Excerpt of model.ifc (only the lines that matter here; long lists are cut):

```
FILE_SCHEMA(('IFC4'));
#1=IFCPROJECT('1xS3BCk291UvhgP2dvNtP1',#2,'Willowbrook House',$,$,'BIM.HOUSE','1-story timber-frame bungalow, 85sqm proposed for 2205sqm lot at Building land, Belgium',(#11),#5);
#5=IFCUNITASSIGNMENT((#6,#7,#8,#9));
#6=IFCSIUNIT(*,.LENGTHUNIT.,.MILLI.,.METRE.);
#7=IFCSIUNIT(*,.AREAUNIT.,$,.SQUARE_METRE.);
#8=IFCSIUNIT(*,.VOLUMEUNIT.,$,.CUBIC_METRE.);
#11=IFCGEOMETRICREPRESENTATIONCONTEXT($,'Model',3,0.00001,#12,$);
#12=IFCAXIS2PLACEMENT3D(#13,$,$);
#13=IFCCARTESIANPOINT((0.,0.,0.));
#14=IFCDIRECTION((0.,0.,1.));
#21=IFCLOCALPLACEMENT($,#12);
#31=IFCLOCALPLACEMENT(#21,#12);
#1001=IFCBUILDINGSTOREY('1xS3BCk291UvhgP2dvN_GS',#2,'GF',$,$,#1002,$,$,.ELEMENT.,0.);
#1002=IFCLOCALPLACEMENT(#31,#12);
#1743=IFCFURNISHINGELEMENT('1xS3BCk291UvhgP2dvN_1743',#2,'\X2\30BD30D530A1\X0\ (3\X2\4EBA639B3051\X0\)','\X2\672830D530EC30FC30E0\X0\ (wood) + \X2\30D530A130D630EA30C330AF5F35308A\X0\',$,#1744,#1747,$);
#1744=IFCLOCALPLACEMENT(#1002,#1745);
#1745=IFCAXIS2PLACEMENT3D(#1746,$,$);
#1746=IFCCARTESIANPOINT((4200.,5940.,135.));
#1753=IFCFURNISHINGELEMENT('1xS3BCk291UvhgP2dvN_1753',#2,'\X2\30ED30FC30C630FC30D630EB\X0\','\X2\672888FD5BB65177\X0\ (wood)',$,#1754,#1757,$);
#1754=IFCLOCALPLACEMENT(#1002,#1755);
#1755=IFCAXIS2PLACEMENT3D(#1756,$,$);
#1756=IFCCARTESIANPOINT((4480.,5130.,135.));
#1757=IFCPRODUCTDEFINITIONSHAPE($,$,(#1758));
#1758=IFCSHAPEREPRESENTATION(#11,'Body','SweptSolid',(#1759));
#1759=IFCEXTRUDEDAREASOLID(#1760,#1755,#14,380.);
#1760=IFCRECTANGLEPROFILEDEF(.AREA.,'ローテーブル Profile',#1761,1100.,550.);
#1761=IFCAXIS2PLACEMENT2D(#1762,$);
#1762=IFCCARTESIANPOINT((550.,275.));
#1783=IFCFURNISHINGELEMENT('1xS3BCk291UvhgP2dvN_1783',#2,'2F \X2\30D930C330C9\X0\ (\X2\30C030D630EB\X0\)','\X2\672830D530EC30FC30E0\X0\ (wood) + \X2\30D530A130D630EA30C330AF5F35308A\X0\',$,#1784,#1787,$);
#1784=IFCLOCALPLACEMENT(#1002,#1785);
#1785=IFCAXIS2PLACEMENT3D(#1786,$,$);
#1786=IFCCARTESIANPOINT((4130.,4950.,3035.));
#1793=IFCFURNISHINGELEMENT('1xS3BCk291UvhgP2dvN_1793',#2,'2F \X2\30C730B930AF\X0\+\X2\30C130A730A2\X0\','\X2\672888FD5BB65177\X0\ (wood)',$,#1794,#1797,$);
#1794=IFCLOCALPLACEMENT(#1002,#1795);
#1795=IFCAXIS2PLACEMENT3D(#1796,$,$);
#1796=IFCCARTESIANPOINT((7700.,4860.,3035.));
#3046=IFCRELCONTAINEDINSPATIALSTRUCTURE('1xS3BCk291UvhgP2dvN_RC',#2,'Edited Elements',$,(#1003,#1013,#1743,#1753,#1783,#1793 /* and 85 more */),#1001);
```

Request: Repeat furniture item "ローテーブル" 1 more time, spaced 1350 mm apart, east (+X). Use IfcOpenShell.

```python
import numpy as np
import ifcopenshell
import ifcopenshell.api.geometry
import ifcopenshell.api.root
import ifcopenshell.util.element
import ifcopenshell.util.placement

model = ifcopenshell.open("model.ifc")


def reuse_history(source, copy):
    """copy_class also copies each property set's owner history, people and application; keep the originals."""
    for rel in copy.IsDefinedBy:
        if rel.is_a("IfcRelDefinesByProperties") and (history := rel.RelatingPropertyDefinition.OwnerHistory):
            rel.RelatingPropertyDefinition.OwnerHistory = source.OwnerHistory
            ifcopenshell.util.element.remove_deep2(model, history)


source = model.by_guid("1xS3BCk291UvhgP2dvN_1753")
base = ifcopenshell.util.placement.get_local_placement(source.ObjectPlacement)
step = np.array([1.0, 0.0, 0.0]) * 1350.0

for i in range(1, 2):
    copy = ifcopenshell.api.root.copy_class(model, product=source)
    copy.Representation = ifcopenshell.util.element.copy_deep(
        model, source.Representation, exclude=["IfcGeometricRepresentationContext", "IfcRepresentationMap"]
    )
    reuse_history(source, copy)
    matrix = base.copy()
    matrix[:3, 3] += i * step
    print("added at", matrix[:3, 3].round(3) + 0.0)
    ifcopenshell.api.geometry.edit_object_placement(model, product=copy, matrix=matrix, is_si=False)

model.write("model_rev.ifc")
```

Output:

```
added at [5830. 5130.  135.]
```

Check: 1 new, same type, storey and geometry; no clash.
